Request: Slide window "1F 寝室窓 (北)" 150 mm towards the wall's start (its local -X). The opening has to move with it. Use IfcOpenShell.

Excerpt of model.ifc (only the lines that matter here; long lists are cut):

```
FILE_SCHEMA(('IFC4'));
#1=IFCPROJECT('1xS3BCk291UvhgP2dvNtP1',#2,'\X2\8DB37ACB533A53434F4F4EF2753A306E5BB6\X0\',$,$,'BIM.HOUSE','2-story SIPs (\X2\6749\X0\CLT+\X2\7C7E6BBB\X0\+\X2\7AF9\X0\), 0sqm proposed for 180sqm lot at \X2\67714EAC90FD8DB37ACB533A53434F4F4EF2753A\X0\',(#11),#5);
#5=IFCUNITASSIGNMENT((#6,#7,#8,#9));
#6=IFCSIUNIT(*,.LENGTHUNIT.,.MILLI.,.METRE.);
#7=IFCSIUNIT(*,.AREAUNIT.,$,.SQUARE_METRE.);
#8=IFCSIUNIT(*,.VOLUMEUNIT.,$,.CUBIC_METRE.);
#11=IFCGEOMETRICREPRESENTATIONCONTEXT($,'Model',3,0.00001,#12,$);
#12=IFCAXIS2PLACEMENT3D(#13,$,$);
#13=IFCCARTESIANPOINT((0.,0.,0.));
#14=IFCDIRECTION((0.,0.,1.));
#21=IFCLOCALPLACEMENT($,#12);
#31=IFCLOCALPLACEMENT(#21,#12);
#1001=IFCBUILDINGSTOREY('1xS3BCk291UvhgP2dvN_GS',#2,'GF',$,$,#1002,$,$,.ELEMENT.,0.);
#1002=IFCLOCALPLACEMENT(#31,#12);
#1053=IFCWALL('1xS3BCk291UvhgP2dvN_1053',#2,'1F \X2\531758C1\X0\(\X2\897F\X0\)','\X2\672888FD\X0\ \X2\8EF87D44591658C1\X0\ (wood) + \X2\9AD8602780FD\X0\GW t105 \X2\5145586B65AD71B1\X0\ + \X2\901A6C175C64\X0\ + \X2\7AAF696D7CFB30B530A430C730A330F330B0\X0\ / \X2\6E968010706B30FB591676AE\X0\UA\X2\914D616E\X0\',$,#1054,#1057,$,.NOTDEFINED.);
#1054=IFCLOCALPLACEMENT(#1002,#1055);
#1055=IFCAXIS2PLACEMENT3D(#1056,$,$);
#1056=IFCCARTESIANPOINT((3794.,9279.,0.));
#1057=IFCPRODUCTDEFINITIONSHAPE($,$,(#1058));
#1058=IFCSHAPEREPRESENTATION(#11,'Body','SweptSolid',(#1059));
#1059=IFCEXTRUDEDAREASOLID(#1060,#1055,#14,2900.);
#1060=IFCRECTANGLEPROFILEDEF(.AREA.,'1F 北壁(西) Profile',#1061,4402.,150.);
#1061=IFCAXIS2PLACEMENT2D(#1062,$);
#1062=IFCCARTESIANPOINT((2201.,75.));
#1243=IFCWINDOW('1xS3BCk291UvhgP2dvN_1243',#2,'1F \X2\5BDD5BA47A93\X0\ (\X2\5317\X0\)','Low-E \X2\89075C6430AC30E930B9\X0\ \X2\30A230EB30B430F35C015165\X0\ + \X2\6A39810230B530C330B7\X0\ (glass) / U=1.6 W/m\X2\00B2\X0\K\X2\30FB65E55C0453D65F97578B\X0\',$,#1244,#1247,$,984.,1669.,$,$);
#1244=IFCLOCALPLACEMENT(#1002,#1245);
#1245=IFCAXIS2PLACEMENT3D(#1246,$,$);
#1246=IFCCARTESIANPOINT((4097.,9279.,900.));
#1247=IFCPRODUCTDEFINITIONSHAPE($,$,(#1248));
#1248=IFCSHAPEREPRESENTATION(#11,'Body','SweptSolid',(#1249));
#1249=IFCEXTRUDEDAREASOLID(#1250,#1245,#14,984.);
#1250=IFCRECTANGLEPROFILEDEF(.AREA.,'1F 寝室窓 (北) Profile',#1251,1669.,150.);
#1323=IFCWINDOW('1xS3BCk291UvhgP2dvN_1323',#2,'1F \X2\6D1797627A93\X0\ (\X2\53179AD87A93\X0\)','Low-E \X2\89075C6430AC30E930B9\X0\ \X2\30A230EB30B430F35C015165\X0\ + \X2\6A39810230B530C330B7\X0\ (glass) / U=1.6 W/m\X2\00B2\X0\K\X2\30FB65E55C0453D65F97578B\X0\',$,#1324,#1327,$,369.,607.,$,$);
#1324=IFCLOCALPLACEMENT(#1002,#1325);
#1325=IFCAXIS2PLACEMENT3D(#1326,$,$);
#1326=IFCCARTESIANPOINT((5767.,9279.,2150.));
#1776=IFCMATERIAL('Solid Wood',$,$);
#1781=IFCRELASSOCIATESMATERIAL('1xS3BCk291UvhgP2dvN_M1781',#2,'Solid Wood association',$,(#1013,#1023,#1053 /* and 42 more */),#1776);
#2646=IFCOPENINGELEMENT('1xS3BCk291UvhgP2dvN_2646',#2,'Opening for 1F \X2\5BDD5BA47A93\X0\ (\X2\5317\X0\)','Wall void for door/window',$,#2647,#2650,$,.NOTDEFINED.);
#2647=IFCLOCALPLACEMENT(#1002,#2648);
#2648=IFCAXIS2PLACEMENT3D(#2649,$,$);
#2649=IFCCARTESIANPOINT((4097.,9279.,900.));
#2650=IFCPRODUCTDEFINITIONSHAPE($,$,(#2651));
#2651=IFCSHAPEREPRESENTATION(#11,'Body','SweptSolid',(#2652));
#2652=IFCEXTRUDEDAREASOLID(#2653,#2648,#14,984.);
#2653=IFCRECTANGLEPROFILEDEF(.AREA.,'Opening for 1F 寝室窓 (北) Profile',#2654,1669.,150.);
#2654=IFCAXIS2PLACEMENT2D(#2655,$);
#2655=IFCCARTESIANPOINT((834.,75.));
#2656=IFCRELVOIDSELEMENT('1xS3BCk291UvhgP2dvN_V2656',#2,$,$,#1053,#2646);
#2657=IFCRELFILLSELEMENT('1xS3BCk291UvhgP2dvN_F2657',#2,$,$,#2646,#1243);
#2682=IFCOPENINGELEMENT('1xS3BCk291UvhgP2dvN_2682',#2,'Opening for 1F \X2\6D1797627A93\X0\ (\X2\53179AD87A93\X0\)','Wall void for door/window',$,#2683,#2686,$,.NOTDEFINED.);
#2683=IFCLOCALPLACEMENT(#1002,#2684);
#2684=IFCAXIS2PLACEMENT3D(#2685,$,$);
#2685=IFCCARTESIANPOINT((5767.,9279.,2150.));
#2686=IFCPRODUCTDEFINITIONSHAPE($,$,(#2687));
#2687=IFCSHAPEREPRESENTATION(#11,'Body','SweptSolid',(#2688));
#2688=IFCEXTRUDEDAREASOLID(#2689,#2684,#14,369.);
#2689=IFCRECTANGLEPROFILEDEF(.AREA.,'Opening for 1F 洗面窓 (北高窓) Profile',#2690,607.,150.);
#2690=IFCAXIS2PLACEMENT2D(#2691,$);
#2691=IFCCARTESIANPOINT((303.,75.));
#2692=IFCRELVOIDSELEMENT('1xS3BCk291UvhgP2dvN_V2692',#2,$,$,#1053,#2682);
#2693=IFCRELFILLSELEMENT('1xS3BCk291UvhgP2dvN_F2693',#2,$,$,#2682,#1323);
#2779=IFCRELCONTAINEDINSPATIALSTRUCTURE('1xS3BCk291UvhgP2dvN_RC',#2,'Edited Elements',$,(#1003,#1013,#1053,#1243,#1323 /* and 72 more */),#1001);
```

```python
import ifcopenshell
import ifcopenshell.api.geometry
import ifcopenshell.util.placement
import ifcopenshell.util.unit

model = ifcopenshell.open("model.ifc")
unit_scale = ifcopenshell.util.unit.calculate_unit_scale(model)

window = model.by_guid("1xS3BCk291UvhgP2dvN_1243")
opening = window.FillsVoids[0].RelatingOpeningElement
wall = opening.VoidsElements[0].RelatingBuildingElement

wall_matrix = ifcopenshell.util.placement.get_local_placement(wall.ObjectPlacement)
shift = wall_matrix[:3, 0] * -0.15 / unit_scale
before = ifcopenshell.util.placement.get_local_placement(window.ObjectPlacement)[:3, 3].copy()

# The window is not placed relative to its opening, so move both.
for product in (opening, window):
    matrix = ifcopenshell.util.placement.get_local_placement(product.ObjectPlacement)
    matrix[:3, 3] += shift
    ifcopenshell.api.geometry.edit_object_placement(model, product=product, matrix=matrix, is_si=False)

after = ifcopenshell.util.placement.get_local_placement(window.ObjectPlacement)[:3, 3]
print("window moved by", (after - before).round(3) + 0.0)

model.write("model_v2.ifc")
```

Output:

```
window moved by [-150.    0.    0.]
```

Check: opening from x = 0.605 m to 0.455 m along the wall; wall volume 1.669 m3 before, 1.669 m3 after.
